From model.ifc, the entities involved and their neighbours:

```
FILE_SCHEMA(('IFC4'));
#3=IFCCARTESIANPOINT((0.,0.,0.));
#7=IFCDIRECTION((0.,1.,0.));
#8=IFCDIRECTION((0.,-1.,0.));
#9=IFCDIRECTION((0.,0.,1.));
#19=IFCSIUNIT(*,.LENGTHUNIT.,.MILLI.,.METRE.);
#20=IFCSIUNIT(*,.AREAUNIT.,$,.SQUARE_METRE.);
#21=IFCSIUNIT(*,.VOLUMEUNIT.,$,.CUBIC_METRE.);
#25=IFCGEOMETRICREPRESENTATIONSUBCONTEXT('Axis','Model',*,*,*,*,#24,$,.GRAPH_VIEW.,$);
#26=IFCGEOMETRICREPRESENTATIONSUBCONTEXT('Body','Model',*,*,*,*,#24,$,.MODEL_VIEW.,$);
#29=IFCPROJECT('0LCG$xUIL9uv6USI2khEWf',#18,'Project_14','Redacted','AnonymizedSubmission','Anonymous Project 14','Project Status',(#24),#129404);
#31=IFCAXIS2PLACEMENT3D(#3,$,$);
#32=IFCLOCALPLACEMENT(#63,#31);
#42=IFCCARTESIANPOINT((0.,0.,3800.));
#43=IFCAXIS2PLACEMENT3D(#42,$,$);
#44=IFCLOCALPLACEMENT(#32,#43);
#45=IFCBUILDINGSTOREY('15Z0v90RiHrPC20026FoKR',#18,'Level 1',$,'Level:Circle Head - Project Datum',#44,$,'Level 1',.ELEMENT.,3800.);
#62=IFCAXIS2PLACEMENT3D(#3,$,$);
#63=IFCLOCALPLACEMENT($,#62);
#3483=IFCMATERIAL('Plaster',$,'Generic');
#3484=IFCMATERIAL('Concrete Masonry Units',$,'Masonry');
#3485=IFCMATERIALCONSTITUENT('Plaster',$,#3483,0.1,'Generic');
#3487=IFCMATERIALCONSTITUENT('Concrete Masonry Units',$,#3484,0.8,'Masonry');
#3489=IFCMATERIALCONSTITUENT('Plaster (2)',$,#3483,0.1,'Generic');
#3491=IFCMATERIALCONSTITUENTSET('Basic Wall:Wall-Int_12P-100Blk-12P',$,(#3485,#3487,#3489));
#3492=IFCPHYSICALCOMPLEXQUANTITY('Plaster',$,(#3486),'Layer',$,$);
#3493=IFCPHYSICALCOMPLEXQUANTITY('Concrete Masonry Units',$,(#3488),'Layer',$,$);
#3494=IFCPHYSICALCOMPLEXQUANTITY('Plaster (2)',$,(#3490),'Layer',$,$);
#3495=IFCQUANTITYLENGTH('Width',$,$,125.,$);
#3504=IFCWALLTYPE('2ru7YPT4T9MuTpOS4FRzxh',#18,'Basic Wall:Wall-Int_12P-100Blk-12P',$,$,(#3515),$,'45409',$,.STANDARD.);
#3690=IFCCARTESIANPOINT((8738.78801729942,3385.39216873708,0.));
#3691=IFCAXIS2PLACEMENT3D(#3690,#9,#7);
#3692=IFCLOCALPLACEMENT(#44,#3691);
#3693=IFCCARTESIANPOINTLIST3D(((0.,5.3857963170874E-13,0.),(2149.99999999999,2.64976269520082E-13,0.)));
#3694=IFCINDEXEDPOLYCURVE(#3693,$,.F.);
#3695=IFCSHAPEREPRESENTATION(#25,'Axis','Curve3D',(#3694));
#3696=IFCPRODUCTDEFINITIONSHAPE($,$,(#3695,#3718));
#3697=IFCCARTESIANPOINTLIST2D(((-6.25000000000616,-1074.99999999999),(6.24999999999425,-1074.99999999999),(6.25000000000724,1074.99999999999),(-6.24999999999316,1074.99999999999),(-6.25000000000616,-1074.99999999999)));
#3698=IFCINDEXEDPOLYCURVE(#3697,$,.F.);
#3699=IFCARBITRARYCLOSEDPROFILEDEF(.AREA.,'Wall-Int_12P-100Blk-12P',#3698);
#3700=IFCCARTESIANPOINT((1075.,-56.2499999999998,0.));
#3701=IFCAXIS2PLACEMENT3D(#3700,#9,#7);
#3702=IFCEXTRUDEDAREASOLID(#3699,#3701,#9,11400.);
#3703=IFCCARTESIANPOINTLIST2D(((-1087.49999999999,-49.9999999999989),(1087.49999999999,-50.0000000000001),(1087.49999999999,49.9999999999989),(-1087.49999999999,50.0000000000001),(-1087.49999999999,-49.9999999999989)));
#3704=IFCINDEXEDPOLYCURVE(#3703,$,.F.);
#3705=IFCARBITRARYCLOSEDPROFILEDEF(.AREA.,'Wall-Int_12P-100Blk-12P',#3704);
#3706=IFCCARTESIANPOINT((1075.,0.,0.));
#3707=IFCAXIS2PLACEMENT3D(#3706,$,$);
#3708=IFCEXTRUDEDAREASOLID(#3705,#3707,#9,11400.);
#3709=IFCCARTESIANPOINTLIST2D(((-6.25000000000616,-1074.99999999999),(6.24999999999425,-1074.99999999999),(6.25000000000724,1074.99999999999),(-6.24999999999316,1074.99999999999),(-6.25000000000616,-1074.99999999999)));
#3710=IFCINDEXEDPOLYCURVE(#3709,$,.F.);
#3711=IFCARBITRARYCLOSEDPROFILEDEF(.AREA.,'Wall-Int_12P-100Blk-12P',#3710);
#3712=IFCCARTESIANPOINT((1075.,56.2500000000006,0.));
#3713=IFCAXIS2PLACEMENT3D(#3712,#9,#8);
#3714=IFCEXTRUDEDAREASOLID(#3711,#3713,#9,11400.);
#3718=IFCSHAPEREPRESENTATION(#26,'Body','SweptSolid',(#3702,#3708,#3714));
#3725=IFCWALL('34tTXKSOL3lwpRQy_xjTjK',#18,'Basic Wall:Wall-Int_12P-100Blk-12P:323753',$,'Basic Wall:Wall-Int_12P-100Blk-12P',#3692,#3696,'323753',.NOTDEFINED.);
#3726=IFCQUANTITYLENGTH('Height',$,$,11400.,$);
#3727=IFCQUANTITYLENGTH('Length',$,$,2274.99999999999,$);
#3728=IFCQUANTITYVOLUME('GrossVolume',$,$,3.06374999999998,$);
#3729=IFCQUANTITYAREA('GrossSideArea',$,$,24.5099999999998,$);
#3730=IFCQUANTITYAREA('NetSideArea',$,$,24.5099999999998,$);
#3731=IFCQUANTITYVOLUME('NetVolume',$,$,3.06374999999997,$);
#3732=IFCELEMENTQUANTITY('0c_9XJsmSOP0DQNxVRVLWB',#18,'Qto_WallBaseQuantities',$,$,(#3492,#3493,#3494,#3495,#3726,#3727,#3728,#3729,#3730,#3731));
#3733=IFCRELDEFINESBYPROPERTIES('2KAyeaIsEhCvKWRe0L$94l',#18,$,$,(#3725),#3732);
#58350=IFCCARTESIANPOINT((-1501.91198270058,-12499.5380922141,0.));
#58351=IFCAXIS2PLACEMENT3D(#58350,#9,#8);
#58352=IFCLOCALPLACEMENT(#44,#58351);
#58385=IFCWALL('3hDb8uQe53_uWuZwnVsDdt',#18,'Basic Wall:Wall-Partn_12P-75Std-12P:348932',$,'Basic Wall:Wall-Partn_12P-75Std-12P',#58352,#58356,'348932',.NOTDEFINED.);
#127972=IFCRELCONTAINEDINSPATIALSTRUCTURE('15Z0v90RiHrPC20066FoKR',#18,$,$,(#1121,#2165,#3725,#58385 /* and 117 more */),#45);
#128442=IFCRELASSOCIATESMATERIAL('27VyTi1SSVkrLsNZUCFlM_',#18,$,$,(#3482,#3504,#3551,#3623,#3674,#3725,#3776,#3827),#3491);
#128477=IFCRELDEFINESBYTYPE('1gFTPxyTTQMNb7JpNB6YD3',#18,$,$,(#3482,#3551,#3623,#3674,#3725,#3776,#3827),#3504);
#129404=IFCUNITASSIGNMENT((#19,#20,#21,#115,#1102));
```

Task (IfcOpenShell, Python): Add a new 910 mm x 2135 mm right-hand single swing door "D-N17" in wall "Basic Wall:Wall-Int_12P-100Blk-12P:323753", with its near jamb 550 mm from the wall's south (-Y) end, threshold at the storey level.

```python
import numpy as np
import ifcopenshell
import ifcopenshell.api.feature
import ifcopenshell.api.geometry
import ifcopenshell.api.pset
import ifcopenshell.api.root
import ifcopenshell.api.spatial
import ifcopenshell.geom
import ifcopenshell.util.element
import ifcopenshell.util.placement
import ifcopenshell.util.representation
import ifcopenshell.util.shape
import ifcopenshell.util.unit

model = ifcopenshell.open("model.ifc")
unit_scale = ifcopenshell.util.unit.calculate_unit_scale(model)
area_scale = ifcopenshell.util.unit.calculate_unit_scale(model, "AREAUNIT")
volume_scale = ifcopenshell.util.unit.calculate_unit_scale(model, "VOLUMEUNIT")
settings = ifcopenshell.geom.settings()


def volume(element):
    """Net volume in cubic metres, openings subtracted."""
    shape = ifcopenshell.geom.create_shape(settings, element)
    return ifcopenshell.util.shape.get_volume(shape.geometry)


wall = model.by_id(3725)
storey = ifcopenshell.util.element.get_container(wall, ifc_class="IfcBuildingStorey")
context = ifcopenshell.util.representation.get_context(model, "Model", "Body", "MODEL_VIEW")
before = volume(wall)

width, height, from_end, sill = 0.91, 2.135, 0.55, 0.0  # metres

# The wall runs along its own X axis, and the end named is its -X end.
wall_shape = ifcopenshell.geom.create_shape(settings, wall)
x, y, z = ifcopenshell.util.shape.get_vertices(wall_shape.geometry).T
start = x.min() + from_end
face, thickness = float(y.min()), float(y.max() - y.min())
wall_matrix = ifcopenshell.util.placement.get_local_placement(wall.ObjectPlacement)
level = ifcopenshell.util.placement.get_local_placement(storey.ObjectPlacement)[2, 3]


def in_wall(x, y):
    """Placement at x, y metres in the wall's axes, at sill height."""
    matrix = wall_matrix.copy()
    matrix[:, 3] = wall_matrix @ np.array([x / unit_scale, y / unit_scale, 0.0, 1.0])
    matrix[2, 3] = level + sill / unit_scale
    return matrix


# Opening: a box that overshoots both wall faces by 50 mm.
opening = ifcopenshell.api.root.create_entity(model, ifc_class="IfcOpeningElement", predefined_type="OPENING")
box = ifcopenshell.api.geometry.add_wall_representation(
    model, context=context, length=width, height=height, thickness=thickness + 0.1
)
ifcopenshell.api.geometry.assign_representation(model, product=opening, representation=box)
ifcopenshell.api.geometry.edit_object_placement(model, product=opening, matrix=in_wall(start, face - 0.05), is_si=False)
ifcopenshell.api.feature.add_feature(model, feature=opening, element=wall)

door = ifcopenshell.api.root.create_entity(model, ifc_class="IfcDoor", name="D-N17", predefined_type="DOOR")
door.OverallWidth, door.OverallHeight = width / unit_scale, height / unit_scale
door.OperationType = "SINGLE_SWING_RIGHT"
body = ifcopenshell.api.geometry.add_door_representation(
    model,
    context=context,
    overall_width=door.OverallWidth,
    overall_height=door.OverallHeight,
    operation_type="SINGLE_SWING_RIGHT",
    lining_properties={"LiningDepth": thickness / unit_scale, "ThresholdDepth": thickness / unit_scale},
)
ifcopenshell.api.geometry.assign_representation(model, product=door, representation=body)
ifcopenshell.api.spatial.assign_container(model, products=[door], relating_structure=storey)
ifcopenshell.api.feature.add_filling(model, opening=opening, element=door)

# The lining spans the wall, so the door starts at the wall face.
ifcopenshell.api.geometry.edit_object_placement(model, product=door, matrix=in_wall(start, face), is_si=False)

after = volume(wall)

# Update the wall's stored quantities.
qto = model.by_id(ifcopenshell.util.element.get_pset(wall, "Qto_WallBaseQuantities", should_inherit=False)["id"])
ifcopenshell.api.pset.edit_qto(model, qto=qto, properties={
    "NetSideArea": after / thickness / area_scale,
    "NetVolume": after / volume_scale,
})

print(f"wall volume {before:.3f} -> {after:.3f} m3")

model.write("model-out.ifc")
```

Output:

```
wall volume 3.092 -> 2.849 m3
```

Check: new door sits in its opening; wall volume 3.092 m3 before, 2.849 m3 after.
